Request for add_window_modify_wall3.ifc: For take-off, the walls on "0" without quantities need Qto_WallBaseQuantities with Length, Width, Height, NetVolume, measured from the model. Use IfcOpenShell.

First a look at what the model holds.

```python
import ifcopenshell
import ifcopenshell.util.element
import ifcopenshell.util.unit

model = ifcopenshell.open("add_window_modify_wall3.ifc")
print(model.schema)
for unit_type in ("LENGTHUNIT", "AREAUNIT", "VOLUMEUNIT"):
    print(unit_type, ifcopenshell.util.unit.calculate_unit_scale(model, unit_type))
storey = next(s for s in model.by_type("IfcBuildingStorey") if s.Name == "0")
walls = [e for e in ifcopenshell.util.element.get_decomposition(storey) if e.is_a("IfcWall")]
for e in sorted(walls, key=lambda e: e.id()):
    print(e.id(), e.is_a(), e.Name, list(ifcopenshell.util.element.get_psets(e, qtos_only=True)), sep=" | ")
```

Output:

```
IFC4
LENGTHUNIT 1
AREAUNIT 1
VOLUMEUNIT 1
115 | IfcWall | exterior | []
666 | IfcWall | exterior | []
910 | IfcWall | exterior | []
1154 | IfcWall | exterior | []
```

```python
import ifcopenshell
import ifcopenshell.api.pset
import ifcopenshell.geom
import ifcopenshell.util.element
import ifcopenshell.util.shape
import ifcopenshell.util.unit

model = ifcopenshell.open("add_window_modify_wall3.ifc")
unit_scale = ifcopenshell.util.unit.calculate_unit_scale(model)
volume_scale = ifcopenshell.util.unit.calculate_unit_scale(model, "VOLUMEUNIT")
settings = ifcopenshell.geom.settings()

storey = next(s for s in model.by_type("IfcBuildingStorey") if s.Name == "0")
walls = [e for e in ifcopenshell.util.element.get_decomposition(storey) if e.is_a("IfcWall")]

for e in sorted(walls, key=lambda e: e.id()):
    if ifcopenshell.util.element.get_psets(e, qtos_only=True, should_inherit=False):
        continue
    # Geometry comes back in metres, in the element's own axes.
    shape = ifcopenshell.geom.create_shape(settings, e)
    values = {
        "Length": ifcopenshell.util.shape.get_x(shape.geometry) / unit_scale,
        "Width": ifcopenshell.util.shape.get_y(shape.geometry) / unit_scale,
        "Height": ifcopenshell.util.shape.get_z(shape.geometry) / unit_scale,
        "NetVolume": ifcopenshell.util.shape.get_volume(shape.geometry) / volume_scale,
    }
    qto = ifcopenshell.api.pset.add_qto(model, product=e, name="Qto_WallBaseQuantities")
    ifcopenshell.api.pset.edit_qto(model, qto=qto, properties=values)
    print(e.id(), {k: round(v, 3) for k, v in values.items()})

model.write("add_window_modify_wall3_edited.ifc")
```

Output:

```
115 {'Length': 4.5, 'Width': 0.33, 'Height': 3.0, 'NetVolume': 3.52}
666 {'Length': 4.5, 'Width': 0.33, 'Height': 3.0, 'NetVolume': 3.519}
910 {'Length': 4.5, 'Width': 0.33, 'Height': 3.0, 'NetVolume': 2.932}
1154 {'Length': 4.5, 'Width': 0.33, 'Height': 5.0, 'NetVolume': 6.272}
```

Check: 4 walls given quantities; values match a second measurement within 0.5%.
